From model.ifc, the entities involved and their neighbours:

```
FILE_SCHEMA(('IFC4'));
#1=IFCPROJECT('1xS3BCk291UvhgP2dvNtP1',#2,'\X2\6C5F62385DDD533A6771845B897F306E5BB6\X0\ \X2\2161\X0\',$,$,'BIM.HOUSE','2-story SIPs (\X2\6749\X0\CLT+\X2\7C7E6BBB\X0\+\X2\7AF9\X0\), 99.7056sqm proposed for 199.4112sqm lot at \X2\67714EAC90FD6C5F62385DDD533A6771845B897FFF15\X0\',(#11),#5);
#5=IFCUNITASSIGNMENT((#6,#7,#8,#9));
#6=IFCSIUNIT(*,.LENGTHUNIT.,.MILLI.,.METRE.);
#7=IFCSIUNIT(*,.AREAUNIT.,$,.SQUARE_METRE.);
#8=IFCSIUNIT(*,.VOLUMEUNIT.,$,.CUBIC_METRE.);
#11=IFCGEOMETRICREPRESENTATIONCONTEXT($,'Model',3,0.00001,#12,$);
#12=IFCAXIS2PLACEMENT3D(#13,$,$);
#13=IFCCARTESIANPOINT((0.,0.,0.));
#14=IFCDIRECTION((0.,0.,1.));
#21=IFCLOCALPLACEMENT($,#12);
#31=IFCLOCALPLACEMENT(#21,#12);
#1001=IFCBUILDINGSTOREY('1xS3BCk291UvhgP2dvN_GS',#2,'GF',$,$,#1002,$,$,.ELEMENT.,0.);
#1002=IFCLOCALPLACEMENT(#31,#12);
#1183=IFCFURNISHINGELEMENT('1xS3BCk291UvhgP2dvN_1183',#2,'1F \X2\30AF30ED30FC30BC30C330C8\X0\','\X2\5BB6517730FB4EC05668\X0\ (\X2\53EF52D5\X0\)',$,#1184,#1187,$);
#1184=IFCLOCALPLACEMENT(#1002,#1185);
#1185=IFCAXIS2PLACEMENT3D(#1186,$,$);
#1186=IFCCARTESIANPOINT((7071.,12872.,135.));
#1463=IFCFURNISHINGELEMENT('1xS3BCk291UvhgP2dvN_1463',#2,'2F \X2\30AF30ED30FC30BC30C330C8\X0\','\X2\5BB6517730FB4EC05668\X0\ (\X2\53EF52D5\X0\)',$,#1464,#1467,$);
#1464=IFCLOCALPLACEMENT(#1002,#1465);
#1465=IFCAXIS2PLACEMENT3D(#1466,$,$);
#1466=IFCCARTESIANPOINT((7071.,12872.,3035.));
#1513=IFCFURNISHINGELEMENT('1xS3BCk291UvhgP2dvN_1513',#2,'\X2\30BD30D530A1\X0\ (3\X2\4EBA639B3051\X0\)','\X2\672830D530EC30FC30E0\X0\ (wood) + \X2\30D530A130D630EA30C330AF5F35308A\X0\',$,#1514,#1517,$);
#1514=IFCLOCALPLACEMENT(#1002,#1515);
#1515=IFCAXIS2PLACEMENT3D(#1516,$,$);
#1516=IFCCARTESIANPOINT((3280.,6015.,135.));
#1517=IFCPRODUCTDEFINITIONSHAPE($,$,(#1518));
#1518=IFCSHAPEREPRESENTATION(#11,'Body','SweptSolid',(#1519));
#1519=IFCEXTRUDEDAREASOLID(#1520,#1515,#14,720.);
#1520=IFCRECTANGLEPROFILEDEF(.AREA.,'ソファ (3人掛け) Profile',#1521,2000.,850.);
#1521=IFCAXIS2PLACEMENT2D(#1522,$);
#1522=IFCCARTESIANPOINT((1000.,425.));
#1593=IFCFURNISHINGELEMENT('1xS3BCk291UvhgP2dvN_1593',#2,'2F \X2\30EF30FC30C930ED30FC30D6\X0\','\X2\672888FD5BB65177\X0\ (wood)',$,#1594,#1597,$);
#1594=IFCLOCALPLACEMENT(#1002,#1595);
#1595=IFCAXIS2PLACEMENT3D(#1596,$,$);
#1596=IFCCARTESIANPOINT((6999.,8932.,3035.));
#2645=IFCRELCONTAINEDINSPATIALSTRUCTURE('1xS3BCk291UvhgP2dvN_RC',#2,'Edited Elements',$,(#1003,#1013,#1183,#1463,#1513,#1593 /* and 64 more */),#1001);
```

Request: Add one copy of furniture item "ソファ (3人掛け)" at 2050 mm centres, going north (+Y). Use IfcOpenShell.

```python
import numpy as np
import ifcopenshell
import ifcopenshell.api.geometry
import ifcopenshell.api.root
import ifcopenshell.util.element
import ifcopenshell.util.placement

model = ifcopenshell.open("model.ifc")


def reuse_history(source, copy):
    """copy_class also copies each property set's owner history, people and application; keep the originals."""
    for rel in copy.IsDefinedBy:
        if rel.is_a("IfcRelDefinesByProperties") and (history := rel.RelatingPropertyDefinition.OwnerHistory):
            rel.RelatingPropertyDefinition.OwnerHistory = source.OwnerHistory
            ifcopenshell.util.element.remove_deep2(model, history)


source = model.by_guid("1xS3BCk291UvhgP2dvN_1513")
base = ifcopenshell.util.placement.get_local_placement(source.ObjectPlacement)
step = np.array([0.0, 1.0, 0.0]) * 2050.0

for i in range(1, 2):
    copy = ifcopenshell.api.root.copy_class(model, product=source)
    copy.Representation = ifcopenshell.util.element.copy_deep(
        model, source.Representation, exclude=["IfcGeometricRepresentationContext", "IfcRepresentationMap"]
    )
    reuse_history(source, copy)
    matrix = base.copy()
    matrix[:3, 3] += i * step
    print("added at", matrix[:3, 3].round(3) + 0.0)
    ifcopenshell.api.geometry.edit_object_placement(model, product=copy, matrix=matrix, is_si=False)

model.write("model_rev.ifc")
```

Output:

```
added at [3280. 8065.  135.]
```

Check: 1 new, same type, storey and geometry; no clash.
